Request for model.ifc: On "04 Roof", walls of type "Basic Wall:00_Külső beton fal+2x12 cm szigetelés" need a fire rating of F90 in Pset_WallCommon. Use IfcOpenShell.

First a look at what the model holds.

```python
import ifcopenshell
import ifcopenshell.util.element

model = ifcopenshell.open("model.ifc")
print(model.schema)
storey = next(s for s in model.by_type("IfcBuildingStorey") if s.Name == "04 Roof")
walls = [e for e in ifcopenshell.util.element.get_decomposition(storey) if e.is_a("IfcWall")]
seen = {}
for e in walls:
    element_type = ifcopenshell.util.element.get_type(e)
    key = (element_type.Name if element_type != e and element_type else None, ifcopenshell.util.element.get_pset(e, "Pset_WallCommon", "FireRating"))
    seen[key] = seen.get(key, 0) + 1
for (name, value), count in sorted(seen.items(), key=str):
    print(count, "x", name, "|", value)
```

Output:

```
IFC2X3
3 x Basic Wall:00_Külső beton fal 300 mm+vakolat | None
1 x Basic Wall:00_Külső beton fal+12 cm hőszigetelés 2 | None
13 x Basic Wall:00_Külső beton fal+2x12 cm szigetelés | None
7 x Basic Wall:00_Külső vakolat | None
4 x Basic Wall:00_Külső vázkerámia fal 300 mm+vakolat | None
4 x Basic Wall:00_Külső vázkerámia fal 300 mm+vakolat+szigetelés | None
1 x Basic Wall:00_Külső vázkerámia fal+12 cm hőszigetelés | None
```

```python
import ifcopenshell
import ifcopenshell.api.pset
import ifcopenshell.util.element

model = ifcopenshell.open("model.ifc")

storey = next(s for s in model.by_type("IfcBuildingStorey") if s.Name == "04 Roof")
walls = [e for e in ifcopenshell.util.element.get_decomposition(storey) if e.is_a("IfcWall")]

count = 0
for e in walls:
    element_type = ifcopenshell.util.element.get_type(e)
    if element_type in (None, e) or element_type.Name != "Basic Wall:00_Külső beton fal+2x12 cm szigetelés":
        continue
    # add_pset returns the element's existing set when there is one.
    pset = ifcopenshell.api.pset.add_pset(model, product=e, name="Pset_WallCommon")
    ifcopenshell.api.pset.edit_pset(model, pset=pset, properties={"FireRating": "F90"})
    count += 1

print(count, "walls updated")

model.write("model_rev.ifc")
```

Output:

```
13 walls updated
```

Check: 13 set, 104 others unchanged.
